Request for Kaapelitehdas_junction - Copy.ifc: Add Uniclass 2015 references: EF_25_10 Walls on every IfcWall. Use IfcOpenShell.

First a look at what the model holds.

```python
import ifcopenshell

model = ifcopenshell.open("Kaapelitehdas_junction - Copy.ifc")
print(model.schema)
print("classifications:", [c.Name for c in model.by_type("IfcClassification")])
for ifc_class in ("IfcDoor", "IfcRoof", "IfcStair", "IfcWall", "IfcWindow"):
    print(ifc_class, len(model.by_type(ifc_class)))
```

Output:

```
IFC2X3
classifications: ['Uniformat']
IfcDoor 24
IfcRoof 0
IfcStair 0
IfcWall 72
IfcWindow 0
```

```python
import ifcopenshell
import ifcopenshell.api.classification

model = ifcopenshell.open("Kaapelitehdas_junction - Copy.ifc")

# IFC2X3 requires Source and Edition and has no link from the project to the system.
system = model.create_entity("IfcClassification", Source="NBS", Edition="2015", Name="Uniclass 2015")

codes = {
    "IfcWall": ("EF_25_10", "Walls"),
}
for ifc_class, (code, name) in codes.items():
    products = model.by_type(ifc_class)
    ifcopenshell.api.classification.add_reference(
        model, products=products, classification=system, identification=code, name=name
    )
    print(code, len(products))

model.write("Kaapelitehdas_junction - Copy_updated.ifc")
```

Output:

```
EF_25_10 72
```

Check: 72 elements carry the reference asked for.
